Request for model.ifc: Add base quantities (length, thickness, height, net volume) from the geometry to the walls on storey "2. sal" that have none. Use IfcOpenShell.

First a look at what the model holds.

```python
import ifcopenshell
import ifcopenshell.util.element
import ifcopenshell.util.unit

model = ifcopenshell.open("model.ifc")
print(model.schema)
for unit_type in ("LENGTHUNIT", "AREAUNIT", "VOLUMEUNIT"):
    print(unit_type, ifcopenshell.util.unit.calculate_unit_scale(model, unit_type))
storey = next(s for s in model.by_type("IfcBuildingStorey") if s.Name == "2. sal")
walls = [e for e in ifcopenshell.util.element.get_decomposition(storey) if e.is_a("IfcWall")]
for e in sorted(walls, key=lambda e: e.id()):
    print(e.id(), e.is_a(), e.Name, list(ifcopenshell.util.element.get_psets(e, qtos_only=True)), sep=" | ")
```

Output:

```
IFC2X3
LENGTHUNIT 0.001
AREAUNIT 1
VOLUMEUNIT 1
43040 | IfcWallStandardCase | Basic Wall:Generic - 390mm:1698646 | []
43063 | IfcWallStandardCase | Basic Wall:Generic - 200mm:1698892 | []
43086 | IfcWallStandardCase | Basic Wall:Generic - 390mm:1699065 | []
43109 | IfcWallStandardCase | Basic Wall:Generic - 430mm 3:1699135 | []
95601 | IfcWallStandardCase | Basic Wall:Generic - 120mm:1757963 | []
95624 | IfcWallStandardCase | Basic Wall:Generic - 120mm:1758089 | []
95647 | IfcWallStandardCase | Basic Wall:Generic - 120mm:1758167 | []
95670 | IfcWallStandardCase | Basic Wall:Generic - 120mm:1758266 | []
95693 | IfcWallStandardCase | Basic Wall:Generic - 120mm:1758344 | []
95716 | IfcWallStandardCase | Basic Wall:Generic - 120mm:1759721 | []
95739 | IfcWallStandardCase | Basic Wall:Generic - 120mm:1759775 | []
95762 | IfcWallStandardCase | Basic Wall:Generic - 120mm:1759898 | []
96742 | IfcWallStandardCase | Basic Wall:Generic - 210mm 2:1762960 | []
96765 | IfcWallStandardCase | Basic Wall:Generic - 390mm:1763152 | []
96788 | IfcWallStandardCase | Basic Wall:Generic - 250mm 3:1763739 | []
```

```python
import ifcopenshell
import ifcopenshell.api.pset
import ifcopenshell.geom
import ifcopenshell.util.element
import ifcopenshell.util.shape
import ifcopenshell.util.unit

model = ifcopenshell.open("model.ifc")
unit_scale = ifcopenshell.util.unit.calculate_unit_scale(model)
volume_scale = ifcopenshell.util.unit.calculate_unit_scale(model, "VOLUMEUNIT")
settings = ifcopenshell.geom.settings()

storey = next(s for s in model.by_type("IfcBuildingStorey") if s.Name == "2. sal")
walls = [e for e in ifcopenshell.util.element.get_decomposition(storey) if e.is_a("IfcWall")]

for e in sorted(walls, key=lambda e: e.id()):
    if ifcopenshell.util.element.get_psets(e, qtos_only=True, should_inherit=False):
        continue
    # Geometry comes back in metres, in the element's own axes.
    shape = ifcopenshell.geom.create_shape(settings, e)
    values = {
        "Length": ifcopenshell.util.shape.get_x(shape.geometry) / unit_scale,
        "Width": ifcopenshell.util.shape.get_y(shape.geometry) / unit_scale,
        "Height": ifcopenshell.util.shape.get_z(shape.geometry) / unit_scale,
        "NetVolume": ifcopenshell.util.shape.get_volume(shape.geometry) / volume_scale,
    }
    qto = ifcopenshell.api.pset.add_qto(model, product=e, name="BaseQuantities")
    ifcopenshell.api.pset.edit_qto(model, qto=qto, properties=values)
    print(e.id(), {k: round(v, 3) for k, v in values.items()})

model.write("model-out.ifc")
```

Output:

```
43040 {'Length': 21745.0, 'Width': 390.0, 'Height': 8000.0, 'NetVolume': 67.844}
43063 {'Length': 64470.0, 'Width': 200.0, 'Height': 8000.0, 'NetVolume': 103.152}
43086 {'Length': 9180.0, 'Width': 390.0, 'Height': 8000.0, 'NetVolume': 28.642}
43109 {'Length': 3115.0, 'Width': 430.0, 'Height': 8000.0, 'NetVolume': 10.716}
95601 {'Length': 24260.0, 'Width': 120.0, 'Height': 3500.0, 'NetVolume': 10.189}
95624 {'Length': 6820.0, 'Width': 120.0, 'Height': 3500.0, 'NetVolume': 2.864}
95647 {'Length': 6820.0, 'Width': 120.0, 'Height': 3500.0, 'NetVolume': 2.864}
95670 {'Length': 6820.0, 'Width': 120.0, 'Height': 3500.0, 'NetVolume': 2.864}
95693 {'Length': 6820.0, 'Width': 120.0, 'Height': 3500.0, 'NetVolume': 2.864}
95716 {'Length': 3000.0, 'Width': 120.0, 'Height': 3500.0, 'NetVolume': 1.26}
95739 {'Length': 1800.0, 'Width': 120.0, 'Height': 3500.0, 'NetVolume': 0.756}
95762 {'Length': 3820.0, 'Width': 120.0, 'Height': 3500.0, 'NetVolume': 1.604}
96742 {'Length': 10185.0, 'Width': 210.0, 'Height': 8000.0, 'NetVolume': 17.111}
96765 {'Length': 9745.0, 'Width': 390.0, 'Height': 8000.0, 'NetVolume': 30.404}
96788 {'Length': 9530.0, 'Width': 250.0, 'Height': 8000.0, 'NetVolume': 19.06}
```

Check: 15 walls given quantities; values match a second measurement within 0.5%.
